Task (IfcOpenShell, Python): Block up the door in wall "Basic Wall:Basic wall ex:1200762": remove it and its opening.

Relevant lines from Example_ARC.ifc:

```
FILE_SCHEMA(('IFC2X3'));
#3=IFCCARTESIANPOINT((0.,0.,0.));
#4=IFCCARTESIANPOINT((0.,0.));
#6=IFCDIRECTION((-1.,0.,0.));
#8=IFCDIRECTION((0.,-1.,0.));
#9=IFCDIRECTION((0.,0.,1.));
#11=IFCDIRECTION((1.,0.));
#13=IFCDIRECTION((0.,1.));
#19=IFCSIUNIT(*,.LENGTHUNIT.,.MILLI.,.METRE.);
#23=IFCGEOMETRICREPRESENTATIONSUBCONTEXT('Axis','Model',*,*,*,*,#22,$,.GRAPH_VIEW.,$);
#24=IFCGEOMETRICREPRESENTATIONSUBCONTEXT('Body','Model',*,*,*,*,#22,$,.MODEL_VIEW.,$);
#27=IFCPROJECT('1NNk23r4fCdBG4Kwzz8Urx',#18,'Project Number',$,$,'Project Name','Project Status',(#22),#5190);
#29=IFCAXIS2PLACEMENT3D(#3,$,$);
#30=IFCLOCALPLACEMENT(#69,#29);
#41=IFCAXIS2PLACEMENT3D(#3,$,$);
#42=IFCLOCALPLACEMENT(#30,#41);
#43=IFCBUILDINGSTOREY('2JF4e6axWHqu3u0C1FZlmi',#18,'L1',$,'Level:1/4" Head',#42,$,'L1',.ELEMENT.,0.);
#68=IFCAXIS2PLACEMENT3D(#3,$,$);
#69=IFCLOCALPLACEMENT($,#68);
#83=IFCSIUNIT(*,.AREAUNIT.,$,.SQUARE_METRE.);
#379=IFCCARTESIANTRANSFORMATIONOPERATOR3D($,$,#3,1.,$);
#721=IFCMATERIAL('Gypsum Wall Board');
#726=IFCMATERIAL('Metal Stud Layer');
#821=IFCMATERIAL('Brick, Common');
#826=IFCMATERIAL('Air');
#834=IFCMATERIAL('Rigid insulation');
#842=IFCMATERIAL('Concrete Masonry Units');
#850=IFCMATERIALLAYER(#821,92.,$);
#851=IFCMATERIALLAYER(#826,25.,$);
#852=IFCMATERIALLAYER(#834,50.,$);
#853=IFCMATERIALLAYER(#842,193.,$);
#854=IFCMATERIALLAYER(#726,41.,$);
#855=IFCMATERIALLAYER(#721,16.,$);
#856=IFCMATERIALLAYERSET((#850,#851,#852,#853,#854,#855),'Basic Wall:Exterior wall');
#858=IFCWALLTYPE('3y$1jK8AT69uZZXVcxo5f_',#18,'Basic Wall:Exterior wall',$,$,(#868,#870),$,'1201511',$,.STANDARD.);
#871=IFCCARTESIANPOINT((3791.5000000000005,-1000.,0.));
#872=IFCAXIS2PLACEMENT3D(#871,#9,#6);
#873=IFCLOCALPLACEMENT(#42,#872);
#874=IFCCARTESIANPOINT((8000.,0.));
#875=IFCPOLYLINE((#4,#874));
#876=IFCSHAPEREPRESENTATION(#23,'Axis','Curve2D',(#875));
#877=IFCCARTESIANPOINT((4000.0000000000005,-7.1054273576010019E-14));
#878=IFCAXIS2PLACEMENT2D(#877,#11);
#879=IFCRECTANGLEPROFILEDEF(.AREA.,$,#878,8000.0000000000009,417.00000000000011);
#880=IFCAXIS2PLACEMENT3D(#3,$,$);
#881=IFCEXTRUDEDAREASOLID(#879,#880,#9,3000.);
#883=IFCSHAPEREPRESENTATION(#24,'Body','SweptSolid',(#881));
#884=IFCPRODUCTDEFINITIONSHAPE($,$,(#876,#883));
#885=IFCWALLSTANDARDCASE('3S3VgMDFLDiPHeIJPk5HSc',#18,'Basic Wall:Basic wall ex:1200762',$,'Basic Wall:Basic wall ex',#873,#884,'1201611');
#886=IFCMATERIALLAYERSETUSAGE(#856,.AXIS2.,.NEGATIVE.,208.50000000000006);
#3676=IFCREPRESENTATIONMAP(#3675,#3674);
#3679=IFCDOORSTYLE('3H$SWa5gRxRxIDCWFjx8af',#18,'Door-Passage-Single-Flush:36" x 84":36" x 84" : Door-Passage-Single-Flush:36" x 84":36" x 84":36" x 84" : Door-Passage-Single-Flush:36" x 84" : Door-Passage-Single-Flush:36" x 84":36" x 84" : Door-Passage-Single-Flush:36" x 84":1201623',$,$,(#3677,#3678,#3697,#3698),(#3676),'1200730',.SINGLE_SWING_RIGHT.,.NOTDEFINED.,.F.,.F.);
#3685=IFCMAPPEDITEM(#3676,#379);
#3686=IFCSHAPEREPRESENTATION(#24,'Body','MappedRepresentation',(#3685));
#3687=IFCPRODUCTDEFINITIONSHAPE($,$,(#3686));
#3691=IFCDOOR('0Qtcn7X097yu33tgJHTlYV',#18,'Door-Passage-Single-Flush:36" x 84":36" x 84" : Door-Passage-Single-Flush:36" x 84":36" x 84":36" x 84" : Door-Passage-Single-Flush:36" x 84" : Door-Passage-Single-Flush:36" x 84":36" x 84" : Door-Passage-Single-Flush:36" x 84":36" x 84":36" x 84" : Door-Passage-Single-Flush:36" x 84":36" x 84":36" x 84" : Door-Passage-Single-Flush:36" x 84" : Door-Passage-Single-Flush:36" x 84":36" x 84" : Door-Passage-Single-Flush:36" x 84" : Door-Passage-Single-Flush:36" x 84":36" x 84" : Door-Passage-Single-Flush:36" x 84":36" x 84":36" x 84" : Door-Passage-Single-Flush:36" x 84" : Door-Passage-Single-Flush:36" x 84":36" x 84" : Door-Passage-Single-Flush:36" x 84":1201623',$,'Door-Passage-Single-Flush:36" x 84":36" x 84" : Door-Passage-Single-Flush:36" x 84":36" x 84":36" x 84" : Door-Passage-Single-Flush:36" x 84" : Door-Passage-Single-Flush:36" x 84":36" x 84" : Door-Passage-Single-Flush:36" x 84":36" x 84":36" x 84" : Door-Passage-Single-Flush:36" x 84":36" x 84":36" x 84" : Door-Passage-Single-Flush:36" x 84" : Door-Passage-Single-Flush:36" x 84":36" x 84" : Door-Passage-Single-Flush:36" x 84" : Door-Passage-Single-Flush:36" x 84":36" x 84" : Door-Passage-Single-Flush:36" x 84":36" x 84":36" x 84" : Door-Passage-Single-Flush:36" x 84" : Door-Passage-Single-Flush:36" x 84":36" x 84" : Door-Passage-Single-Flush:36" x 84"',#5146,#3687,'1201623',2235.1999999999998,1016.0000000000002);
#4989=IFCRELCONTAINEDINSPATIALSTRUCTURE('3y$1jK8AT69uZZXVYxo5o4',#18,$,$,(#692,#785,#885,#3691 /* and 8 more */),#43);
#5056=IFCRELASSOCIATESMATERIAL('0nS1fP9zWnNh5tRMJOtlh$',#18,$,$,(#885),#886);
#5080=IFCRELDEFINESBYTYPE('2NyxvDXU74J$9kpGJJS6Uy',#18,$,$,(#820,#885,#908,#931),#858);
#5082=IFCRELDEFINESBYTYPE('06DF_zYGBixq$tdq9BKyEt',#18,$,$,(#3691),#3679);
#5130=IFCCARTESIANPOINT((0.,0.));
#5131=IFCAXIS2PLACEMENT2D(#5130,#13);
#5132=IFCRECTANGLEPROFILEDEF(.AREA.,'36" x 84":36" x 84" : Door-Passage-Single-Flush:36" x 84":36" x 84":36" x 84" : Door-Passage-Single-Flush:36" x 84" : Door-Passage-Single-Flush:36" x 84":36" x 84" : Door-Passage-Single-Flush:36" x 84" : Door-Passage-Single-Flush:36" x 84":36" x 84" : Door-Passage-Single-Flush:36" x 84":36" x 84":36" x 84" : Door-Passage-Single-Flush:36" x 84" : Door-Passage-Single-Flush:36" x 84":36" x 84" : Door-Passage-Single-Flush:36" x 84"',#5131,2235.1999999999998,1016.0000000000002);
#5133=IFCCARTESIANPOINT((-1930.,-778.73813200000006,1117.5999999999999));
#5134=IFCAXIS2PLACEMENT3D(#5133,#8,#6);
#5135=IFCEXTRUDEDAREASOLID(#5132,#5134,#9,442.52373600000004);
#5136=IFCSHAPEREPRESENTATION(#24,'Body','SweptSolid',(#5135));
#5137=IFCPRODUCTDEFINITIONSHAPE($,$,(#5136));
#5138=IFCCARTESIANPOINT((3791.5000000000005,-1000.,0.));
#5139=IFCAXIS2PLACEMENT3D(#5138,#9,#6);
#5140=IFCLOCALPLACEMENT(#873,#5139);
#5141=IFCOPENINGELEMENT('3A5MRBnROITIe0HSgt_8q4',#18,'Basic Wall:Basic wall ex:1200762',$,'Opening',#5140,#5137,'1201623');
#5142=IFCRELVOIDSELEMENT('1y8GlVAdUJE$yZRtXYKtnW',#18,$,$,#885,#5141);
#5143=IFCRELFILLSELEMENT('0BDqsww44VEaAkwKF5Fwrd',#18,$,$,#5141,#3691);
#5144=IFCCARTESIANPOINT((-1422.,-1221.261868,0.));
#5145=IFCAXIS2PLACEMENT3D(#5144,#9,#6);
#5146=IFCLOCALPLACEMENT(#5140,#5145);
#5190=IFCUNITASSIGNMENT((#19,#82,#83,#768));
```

```python
import ifcopenshell
import ifcopenshell.api.feature
import ifcopenshell.api.root
import ifcopenshell.geom
import ifcopenshell.util.shape

model = ifcopenshell.open("Example_ARC.ifc")
settings = ifcopenshell.geom.settings()


def volume(element):
    """Net volume in cubic metres, openings subtracted."""
    shape = ifcopenshell.geom.create_shape(settings, element)
    return ifcopenshell.util.shape.get_volume(shape.geometry)


door = model.by_guid("0Qtcn7X097yu33tgJHTlYV")
opening = door.FillsVoids[0].RelatingOpeningElement
wall = opening.VoidsElements[0].RelatingBuildingElement
before = volume(wall)

ifcopenshell.api.root.remove_product(model, product=door)
ifcopenshell.api.feature.remove_feature(model, feature=opening)

after = volume(wall)

print(f"wall volume {before:.3f} -> {after:.3f} m3")

model.write("Example_ARC_v2.ifc")
```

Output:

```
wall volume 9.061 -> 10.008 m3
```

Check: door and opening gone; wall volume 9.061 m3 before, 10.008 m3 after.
